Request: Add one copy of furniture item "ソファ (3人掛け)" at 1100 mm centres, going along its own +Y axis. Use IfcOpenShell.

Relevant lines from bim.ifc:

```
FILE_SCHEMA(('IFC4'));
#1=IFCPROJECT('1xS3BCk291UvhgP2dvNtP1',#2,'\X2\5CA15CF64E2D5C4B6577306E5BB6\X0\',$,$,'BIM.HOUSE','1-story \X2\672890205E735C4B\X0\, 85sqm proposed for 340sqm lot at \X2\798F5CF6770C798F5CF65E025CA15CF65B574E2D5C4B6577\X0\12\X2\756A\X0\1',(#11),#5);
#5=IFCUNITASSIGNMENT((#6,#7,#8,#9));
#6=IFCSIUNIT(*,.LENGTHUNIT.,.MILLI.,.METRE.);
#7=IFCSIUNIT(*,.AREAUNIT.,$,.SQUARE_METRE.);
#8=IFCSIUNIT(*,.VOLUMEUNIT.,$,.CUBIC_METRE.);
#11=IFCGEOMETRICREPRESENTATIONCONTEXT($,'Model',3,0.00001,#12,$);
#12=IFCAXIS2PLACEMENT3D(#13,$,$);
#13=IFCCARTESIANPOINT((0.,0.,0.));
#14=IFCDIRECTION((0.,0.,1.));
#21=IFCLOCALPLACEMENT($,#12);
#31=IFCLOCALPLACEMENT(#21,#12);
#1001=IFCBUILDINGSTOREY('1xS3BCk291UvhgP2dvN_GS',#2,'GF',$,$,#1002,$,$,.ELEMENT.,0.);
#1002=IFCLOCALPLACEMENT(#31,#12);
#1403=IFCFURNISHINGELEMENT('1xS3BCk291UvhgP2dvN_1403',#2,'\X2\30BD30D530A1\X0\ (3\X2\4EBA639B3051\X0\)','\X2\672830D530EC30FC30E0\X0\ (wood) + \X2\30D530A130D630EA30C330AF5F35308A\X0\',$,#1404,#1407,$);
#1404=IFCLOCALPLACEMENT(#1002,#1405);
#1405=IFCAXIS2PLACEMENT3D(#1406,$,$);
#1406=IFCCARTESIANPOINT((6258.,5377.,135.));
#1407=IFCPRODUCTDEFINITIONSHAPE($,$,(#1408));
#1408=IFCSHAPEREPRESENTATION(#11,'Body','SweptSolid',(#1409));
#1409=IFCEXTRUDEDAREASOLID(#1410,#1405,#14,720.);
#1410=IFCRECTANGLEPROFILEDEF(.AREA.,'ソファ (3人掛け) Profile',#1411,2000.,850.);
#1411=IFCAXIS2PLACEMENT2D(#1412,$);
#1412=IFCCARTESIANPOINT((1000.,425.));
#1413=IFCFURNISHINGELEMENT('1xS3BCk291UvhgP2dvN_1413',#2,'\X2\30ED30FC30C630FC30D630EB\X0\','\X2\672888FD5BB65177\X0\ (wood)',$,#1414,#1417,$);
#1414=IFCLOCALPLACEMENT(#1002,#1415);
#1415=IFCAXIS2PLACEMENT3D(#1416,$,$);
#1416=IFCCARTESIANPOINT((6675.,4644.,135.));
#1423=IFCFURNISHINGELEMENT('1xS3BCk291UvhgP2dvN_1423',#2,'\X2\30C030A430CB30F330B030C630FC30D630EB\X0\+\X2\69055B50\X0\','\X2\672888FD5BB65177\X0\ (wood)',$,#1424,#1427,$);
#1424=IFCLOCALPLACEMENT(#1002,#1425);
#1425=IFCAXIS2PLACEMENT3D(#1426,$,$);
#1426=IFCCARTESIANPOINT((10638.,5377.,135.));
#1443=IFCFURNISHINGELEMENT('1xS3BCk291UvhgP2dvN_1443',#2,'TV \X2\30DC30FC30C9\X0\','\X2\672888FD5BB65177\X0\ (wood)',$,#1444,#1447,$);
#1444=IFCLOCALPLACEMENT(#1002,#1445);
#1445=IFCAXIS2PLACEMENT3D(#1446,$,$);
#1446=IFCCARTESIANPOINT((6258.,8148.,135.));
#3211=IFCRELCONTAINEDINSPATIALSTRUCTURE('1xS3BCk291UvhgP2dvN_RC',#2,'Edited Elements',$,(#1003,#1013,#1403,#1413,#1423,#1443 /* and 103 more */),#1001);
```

```python
import ifcopenshell
import ifcopenshell.api.geometry
import ifcopenshell.api.root
import ifcopenshell.util.element
import ifcopenshell.util.placement
import ifcopenshell.util.unit

model = ifcopenshell.open("bim.ifc")
unit_scale = ifcopenshell.util.unit.calculate_unit_scale(model)


def reuse_history(source, copy):
    """copy_class also copies each property set's owner history, people and application; keep the originals."""
    for rel in copy.IsDefinedBy:
        if rel.is_a("IfcRelDefinesByProperties") and (history := rel.RelatingPropertyDefinition.OwnerHistory):
            rel.RelatingPropertyDefinition.OwnerHistory = source.OwnerHistory
            ifcopenshell.util.element.remove_deep2(model, history)


source = model.by_guid("1xS3BCk291UvhgP2dvN_1403")
base = ifcopenshell.util.placement.get_local_placement(source.ObjectPlacement)
step = base[:3, 1] * 1.1 / unit_scale

for i in range(1, 2):
    copy = ifcopenshell.api.root.copy_class(model, product=source)
    copy.Representation = ifcopenshell.util.element.copy_deep(
        model, source.Representation, exclude=["IfcGeometricRepresentationContext", "IfcRepresentationMap"]
    )
    reuse_history(source, copy)
    matrix = base.copy()
    matrix[:3, 3] += i * step
    print("added at", matrix[:3, 3].round(3) + 0.0)
    ifcopenshell.api.geometry.edit_object_placement(model, product=copy, matrix=matrix, is_si=False)

model.write("bim_v2.ifc")
```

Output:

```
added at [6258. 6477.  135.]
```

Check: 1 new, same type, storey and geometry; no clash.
